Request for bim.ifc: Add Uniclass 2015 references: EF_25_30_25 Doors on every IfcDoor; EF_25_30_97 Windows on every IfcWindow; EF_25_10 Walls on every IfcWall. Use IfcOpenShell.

First a look at what the model holds.

```python
import ifcopenshell

model = ifcopenshell.open("bim.ifc")
print(model.schema)
print("classifications:", [c.Name for c in model.by_type("IfcClassification")])
for ifc_class in ("IfcDoor", "IfcRoof", "IfcStair", "IfcWall", "IfcWindow"):
    print(ifc_class, len(model.by_type(ifc_class)))
```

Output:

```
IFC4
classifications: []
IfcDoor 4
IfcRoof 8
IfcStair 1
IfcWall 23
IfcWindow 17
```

```python
import ifcopenshell
import ifcopenshell.api.classification

model = ifcopenshell.open("bim.ifc")

system = ifcopenshell.api.classification.add_classification(model, classification="Uniclass 2015")

codes = {
    "IfcDoor": ("EF_25_30_25", "Doors"),
    "IfcWindow": ("EF_25_30_97", "Windows"),
    "IfcWall": ("EF_25_10", "Walls"),
}
for ifc_class, (code, name) in codes.items():
    products = model.by_type(ifc_class)
    ifcopenshell.api.classification.add_reference(
        model, products=products, classification=system, identification=code, name=name
    )
    print(code, len(products))

model.write("bim_rev.ifc")
```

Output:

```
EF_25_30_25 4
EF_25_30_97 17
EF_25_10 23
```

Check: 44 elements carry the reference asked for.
